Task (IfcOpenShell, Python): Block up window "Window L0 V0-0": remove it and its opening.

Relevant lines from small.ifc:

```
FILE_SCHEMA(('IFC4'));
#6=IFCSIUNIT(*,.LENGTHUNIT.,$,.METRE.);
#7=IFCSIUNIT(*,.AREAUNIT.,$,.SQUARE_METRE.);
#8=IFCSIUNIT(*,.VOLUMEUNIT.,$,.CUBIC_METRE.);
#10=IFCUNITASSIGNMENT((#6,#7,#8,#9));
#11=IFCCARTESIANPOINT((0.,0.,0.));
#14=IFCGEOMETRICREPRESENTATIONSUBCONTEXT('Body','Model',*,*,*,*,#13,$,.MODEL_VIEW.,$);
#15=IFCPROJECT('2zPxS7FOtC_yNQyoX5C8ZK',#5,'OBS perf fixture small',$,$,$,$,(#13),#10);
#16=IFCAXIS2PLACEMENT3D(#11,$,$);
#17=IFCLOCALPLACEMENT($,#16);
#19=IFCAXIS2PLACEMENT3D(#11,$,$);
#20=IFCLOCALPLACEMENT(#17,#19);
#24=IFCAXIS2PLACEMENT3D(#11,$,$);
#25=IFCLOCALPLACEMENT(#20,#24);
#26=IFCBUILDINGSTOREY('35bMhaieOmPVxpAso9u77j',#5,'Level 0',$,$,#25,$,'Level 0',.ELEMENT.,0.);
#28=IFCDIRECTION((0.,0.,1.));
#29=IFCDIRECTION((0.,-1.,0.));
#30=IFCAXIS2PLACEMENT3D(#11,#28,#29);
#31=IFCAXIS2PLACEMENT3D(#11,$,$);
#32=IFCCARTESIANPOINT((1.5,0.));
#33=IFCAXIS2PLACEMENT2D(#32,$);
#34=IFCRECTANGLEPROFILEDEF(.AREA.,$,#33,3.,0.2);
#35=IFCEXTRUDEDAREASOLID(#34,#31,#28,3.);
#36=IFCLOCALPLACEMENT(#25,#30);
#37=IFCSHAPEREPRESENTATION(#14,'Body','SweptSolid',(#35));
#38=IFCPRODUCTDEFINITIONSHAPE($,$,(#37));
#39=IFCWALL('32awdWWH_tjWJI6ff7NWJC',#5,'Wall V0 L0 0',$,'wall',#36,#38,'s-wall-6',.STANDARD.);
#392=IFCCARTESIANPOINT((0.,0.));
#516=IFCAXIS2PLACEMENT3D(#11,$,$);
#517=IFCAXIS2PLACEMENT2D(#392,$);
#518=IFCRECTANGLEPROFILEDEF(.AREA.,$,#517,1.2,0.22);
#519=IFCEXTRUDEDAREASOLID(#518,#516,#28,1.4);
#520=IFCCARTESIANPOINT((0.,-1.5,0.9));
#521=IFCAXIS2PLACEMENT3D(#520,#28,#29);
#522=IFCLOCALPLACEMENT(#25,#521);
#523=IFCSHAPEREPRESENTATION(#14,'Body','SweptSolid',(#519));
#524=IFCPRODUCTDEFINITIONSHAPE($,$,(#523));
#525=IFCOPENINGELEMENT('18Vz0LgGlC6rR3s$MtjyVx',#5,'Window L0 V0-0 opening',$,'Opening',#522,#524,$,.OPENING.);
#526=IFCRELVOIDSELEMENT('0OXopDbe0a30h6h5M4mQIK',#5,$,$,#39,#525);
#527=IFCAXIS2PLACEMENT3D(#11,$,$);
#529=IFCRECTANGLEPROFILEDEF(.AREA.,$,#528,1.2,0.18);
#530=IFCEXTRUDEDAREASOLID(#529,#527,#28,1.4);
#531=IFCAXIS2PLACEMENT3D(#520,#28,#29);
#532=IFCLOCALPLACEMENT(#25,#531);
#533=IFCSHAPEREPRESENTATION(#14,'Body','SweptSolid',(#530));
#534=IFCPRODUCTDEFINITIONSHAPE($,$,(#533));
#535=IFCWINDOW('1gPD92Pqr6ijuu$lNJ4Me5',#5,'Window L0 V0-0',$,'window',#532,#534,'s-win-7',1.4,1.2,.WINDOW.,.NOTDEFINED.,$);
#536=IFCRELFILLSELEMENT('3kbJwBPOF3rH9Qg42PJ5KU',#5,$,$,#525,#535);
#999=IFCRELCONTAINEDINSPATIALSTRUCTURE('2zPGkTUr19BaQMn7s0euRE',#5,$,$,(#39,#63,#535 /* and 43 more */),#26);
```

```python
import ifcopenshell
import ifcopenshell.api.feature
import ifcopenshell.api.root
import ifcopenshell.geom
import ifcopenshell.util.shape

model = ifcopenshell.open("small.ifc")
settings = ifcopenshell.geom.settings()


def volume(element):
    """Net volume in cubic metres, openings subtracted."""
    shape = ifcopenshell.geom.create_shape(settings, element)
    return ifcopenshell.util.shape.get_volume(shape.geometry)


window = model.by_guid("1gPD92Pqr6ijuu$lNJ4Me5")
opening = window.FillsVoids[0].RelatingOpeningElement
wall = opening.VoidsElements[0].RelatingBuildingElement
before = volume(wall)

ifcopenshell.api.root.remove_product(model, product=window)
ifcopenshell.api.feature.remove_feature(model, feature=opening)

after = volume(wall)

print(f"wall volume {before:.3f} -> {after:.3f} m3")

model.write("small-out.ifc")
```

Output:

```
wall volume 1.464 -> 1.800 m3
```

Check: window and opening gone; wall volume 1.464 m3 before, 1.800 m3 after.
